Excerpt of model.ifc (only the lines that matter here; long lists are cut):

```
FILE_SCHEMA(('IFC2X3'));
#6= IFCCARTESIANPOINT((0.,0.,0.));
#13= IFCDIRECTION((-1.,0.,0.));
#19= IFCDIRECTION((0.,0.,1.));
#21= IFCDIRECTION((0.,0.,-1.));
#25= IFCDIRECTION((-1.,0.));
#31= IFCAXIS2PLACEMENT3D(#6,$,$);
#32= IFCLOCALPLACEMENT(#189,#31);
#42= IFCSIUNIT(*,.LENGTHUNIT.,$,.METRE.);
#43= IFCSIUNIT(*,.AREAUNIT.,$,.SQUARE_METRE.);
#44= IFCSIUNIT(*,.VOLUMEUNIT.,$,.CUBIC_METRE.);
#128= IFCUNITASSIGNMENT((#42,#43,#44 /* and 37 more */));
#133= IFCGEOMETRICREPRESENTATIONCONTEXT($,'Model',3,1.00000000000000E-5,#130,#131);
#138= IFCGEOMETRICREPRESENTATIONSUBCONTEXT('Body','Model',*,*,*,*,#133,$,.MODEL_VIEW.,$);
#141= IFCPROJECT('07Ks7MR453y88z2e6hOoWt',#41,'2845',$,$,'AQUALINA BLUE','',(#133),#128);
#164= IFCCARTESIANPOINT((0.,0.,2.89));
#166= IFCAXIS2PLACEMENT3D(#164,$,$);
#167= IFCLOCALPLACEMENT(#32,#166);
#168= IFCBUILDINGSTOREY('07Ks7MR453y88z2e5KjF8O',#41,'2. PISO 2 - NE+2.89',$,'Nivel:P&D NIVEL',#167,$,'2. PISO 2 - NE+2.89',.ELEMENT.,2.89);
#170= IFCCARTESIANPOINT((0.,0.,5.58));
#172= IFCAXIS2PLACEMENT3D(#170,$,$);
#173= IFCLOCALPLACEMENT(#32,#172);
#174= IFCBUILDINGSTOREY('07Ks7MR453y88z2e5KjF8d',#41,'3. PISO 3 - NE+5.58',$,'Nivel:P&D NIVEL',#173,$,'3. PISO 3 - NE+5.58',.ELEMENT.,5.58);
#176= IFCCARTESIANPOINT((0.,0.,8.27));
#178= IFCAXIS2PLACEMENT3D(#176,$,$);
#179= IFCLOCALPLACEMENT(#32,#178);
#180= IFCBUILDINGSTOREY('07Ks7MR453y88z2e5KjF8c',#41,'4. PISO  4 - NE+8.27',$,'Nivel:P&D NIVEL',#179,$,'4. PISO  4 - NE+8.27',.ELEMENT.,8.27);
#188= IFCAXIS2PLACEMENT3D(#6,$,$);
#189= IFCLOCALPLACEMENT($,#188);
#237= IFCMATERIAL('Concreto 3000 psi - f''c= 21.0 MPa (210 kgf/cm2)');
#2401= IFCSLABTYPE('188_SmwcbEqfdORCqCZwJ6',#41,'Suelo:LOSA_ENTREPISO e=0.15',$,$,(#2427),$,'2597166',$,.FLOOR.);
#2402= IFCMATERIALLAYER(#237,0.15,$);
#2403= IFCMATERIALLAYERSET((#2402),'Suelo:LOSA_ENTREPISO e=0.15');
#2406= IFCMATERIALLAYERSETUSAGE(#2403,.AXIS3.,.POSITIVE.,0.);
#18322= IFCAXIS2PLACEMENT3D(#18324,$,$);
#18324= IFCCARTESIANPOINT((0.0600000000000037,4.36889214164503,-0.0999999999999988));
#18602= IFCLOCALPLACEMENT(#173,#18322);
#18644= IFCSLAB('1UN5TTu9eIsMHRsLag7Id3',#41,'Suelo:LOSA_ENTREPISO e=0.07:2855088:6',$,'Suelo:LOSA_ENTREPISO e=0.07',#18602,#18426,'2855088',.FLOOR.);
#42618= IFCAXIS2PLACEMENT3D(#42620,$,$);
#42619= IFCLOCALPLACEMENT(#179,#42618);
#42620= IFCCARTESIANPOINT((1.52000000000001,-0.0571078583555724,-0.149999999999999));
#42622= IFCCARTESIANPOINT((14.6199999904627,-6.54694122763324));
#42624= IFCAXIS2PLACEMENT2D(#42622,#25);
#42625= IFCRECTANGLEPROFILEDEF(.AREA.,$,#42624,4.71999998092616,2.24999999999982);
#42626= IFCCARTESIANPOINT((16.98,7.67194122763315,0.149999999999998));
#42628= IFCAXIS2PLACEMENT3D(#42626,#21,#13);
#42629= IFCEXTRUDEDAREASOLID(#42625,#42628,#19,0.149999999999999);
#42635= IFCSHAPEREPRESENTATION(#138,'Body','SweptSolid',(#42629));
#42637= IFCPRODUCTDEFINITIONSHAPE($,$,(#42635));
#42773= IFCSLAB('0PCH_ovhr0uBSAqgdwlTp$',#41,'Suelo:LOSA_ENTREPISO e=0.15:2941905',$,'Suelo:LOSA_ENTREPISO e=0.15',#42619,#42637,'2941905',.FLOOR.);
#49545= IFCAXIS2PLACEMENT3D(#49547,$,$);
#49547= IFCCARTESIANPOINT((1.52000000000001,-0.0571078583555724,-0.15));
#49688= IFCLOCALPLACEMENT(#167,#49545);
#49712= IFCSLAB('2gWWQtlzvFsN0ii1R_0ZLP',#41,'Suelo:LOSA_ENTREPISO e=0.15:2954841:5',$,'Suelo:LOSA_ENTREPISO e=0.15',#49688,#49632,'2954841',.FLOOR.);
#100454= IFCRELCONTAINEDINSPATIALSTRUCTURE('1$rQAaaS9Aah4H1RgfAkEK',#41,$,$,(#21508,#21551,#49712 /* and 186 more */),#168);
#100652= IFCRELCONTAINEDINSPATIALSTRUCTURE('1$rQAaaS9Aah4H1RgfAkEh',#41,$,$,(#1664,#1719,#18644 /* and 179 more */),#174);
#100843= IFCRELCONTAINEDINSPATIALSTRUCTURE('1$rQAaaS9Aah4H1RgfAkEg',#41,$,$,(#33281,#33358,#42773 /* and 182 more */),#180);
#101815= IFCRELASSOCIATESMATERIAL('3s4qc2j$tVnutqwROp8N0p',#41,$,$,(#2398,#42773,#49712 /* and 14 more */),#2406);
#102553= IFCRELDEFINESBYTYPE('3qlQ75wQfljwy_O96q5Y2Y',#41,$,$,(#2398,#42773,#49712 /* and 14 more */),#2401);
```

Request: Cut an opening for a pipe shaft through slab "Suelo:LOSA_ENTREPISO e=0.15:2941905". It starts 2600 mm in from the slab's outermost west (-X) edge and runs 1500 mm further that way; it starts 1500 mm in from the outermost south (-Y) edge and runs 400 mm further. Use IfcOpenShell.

```python
import numpy as np
import ifcopenshell
import ifcopenshell.api.feature
import ifcopenshell.api.geometry
import ifcopenshell.api.root
import ifcopenshell.geom
import ifcopenshell.util.placement
import ifcopenshell.util.representation
import ifcopenshell.util.shape
import ifcopenshell.util.unit

model = ifcopenshell.open("model.ifc")
unit_scale = ifcopenshell.util.unit.calculate_unit_scale(model)
settings = ifcopenshell.geom.settings()


def volume(element):
    """Net volume in cubic metres, openings subtracted."""
    shape = ifcopenshell.geom.create_shape(settings, element)
    return ifcopenshell.util.shape.get_volume(shape.geometry)


slab = model.by_guid("0PCH_ovhr0uBSAqgdwlTp$")
before = volume(slab)

# Extent in the slab's own axes, in metres. The edges named are its -X and -Y sides.
slab_shape = ifcopenshell.geom.create_shape(settings, slab)
vertices = ifcopenshell.util.shape.get_vertices(slab_shape.geometry)
x_min, y_min, bottom = vertices.min(axis=0)
top = vertices[:, 2].max()

opening = ifcopenshell.api.root.create_entity(model, ifc_class="IfcOpeningElement", name="Pipe shaft opening")
context = ifcopenshell.util.representation.get_context(model, "Model", "Body", "MODEL_VIEW")
width, depth = 1.5, 0.4
outline = [(0.0, 0.0), (width, 0.0), (width, depth), (0.0, depth), (0.0, 0.0)]
# Overshoot both faces by 50 mm so the cut is clean.
shape = ifcopenshell.api.geometry.add_slab_representation(
    model, context=context, depth=top - bottom + 0.1, polyline=outline
)
ifcopenshell.api.geometry.assign_representation(model, product=opening, representation=shape)

matrix = ifcopenshell.util.placement.get_local_placement(slab.ObjectPlacement)
matrix[:, 3] = matrix @ np.append(np.array([x_min + 2.6, y_min + 1.5, bottom - 0.05]) / unit_scale, 1.0)
ifcopenshell.api.geometry.edit_object_placement(model, product=opening, matrix=matrix, is_si=False)
ifcopenshell.api.feature.add_feature(model, feature=opening, element=slab)

after = volume(slab)

print(f"slab volume {before:.3f} -> {after:.3f} m3")

model.write("model_updated.ifc")
```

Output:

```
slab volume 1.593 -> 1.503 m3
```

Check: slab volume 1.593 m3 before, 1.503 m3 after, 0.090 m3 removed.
